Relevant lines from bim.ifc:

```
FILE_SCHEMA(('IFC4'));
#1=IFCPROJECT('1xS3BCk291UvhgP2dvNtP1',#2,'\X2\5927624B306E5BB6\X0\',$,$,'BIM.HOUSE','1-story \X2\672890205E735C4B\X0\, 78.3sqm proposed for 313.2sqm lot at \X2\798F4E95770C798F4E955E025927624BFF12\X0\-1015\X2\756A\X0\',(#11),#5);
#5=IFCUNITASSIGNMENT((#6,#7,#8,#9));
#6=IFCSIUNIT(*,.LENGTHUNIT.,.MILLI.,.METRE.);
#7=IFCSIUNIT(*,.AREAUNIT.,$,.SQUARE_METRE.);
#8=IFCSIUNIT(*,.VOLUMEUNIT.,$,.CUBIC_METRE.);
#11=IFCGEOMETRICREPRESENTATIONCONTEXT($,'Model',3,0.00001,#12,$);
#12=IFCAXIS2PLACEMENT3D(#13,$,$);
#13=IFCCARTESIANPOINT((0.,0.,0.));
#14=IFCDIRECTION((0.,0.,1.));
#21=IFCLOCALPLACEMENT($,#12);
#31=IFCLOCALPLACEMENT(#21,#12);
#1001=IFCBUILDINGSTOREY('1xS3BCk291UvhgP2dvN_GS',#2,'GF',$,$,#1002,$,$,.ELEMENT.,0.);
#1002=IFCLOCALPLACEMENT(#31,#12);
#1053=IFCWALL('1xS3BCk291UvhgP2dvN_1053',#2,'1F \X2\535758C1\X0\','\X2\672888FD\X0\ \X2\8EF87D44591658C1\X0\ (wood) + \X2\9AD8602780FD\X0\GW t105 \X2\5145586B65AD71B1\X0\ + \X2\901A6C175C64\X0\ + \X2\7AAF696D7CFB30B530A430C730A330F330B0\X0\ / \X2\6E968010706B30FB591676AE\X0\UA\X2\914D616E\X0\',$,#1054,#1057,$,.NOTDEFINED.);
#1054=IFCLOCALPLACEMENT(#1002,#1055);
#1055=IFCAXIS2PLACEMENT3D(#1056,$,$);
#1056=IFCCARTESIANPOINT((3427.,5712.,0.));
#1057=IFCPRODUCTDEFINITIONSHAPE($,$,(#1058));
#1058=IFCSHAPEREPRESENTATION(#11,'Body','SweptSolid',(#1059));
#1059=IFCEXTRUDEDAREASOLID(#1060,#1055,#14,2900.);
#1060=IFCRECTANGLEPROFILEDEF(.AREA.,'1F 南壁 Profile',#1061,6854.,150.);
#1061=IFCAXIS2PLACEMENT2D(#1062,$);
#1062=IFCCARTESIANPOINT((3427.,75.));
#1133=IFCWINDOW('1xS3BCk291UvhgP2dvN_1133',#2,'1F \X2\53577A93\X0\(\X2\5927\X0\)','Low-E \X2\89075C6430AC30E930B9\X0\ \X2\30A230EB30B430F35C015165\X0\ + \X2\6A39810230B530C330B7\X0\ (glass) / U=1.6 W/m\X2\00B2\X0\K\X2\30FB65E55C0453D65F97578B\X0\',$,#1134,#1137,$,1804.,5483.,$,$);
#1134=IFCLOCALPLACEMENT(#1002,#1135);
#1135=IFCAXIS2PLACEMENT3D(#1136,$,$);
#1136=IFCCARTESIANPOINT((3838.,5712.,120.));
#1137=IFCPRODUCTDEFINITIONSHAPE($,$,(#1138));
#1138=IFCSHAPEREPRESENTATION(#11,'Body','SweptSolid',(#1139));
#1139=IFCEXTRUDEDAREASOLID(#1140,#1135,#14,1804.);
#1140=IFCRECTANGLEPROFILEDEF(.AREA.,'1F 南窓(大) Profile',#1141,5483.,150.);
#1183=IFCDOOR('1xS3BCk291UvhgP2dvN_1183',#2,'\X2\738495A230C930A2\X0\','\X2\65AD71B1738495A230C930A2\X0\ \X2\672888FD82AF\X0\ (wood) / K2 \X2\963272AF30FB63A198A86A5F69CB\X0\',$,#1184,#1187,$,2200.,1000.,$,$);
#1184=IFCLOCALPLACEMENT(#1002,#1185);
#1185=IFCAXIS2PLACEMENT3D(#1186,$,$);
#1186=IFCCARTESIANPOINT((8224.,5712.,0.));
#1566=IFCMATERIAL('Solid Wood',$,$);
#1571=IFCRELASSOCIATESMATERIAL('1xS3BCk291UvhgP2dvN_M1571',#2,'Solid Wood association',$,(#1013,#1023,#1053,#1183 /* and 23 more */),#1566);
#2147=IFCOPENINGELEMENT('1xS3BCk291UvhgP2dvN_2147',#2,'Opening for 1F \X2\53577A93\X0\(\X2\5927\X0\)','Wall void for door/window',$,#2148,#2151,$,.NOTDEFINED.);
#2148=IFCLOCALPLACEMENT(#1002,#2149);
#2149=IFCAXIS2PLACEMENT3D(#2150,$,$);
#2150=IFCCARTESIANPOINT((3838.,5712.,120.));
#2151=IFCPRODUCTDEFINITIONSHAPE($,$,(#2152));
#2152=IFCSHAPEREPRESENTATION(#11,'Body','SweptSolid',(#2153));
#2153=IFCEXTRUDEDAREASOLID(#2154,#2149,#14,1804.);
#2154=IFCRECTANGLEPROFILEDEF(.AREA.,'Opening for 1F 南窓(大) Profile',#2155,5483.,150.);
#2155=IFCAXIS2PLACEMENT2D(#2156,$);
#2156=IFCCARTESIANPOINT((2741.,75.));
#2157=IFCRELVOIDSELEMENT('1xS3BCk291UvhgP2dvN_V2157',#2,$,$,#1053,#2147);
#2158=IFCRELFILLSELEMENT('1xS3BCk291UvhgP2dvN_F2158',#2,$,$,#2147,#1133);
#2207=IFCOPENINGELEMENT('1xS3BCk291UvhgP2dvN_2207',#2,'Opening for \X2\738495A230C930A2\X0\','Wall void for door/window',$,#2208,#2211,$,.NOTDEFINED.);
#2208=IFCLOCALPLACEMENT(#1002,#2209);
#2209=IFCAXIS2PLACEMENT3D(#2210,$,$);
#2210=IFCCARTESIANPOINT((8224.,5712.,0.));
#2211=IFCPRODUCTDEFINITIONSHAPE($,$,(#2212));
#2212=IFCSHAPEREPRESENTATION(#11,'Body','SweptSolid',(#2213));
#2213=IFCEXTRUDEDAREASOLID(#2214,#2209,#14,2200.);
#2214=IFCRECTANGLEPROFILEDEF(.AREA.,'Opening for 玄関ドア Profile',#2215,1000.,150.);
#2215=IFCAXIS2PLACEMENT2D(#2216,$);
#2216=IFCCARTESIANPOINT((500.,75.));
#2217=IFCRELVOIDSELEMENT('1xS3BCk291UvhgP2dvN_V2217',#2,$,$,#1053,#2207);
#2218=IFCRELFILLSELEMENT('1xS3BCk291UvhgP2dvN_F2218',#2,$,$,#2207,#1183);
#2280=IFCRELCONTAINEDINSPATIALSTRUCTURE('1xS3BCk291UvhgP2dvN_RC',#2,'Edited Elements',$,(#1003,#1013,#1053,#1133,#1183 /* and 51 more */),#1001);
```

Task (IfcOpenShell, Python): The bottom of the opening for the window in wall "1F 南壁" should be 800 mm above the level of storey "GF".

```python
import numpy as np
import ifcopenshell
import ifcopenshell.api.geometry
import ifcopenshell.geom
import ifcopenshell.util.element
import ifcopenshell.util.placement
import ifcopenshell.util.shape
import ifcopenshell.util.unit

model = ifcopenshell.open("bim.ifc")
unit_scale = ifcopenshell.util.unit.calculate_unit_scale(model)

window = model.by_guid("1xS3BCk291UvhgP2dvN_1133")
opening = window.FillsVoids[0].RelatingOpeningElement
storey = ifcopenshell.util.element.get_container(window, ifc_class="IfcBuildingStorey")
level = ifcopenshell.util.placement.get_local_placement(storey.ObjectPlacement)[2, 3]

# The opening's origin need not be at the sill, so measure its lowest point.
shape = ifcopenshell.geom.create_shape(ifcopenshell.geom.settings(), opening)
bottom = ifcopenshell.util.shape.get_shape_bottom_elevation(shape, shape.geometry) / unit_scale
dz = level + 0.8 / unit_scale - bottom

shift = np.array([0.0, 0.0, dz])
# The window is not placed relative to its opening, so move both.
for product in (opening, window):
    matrix = ifcopenshell.util.placement.get_local_placement(product.ObjectPlacement)
    matrix[:3, 3] += shift
    ifcopenshell.api.geometry.edit_object_placement(model, product=product, matrix=matrix, is_si=False)

print(f"moved by {dz * unit_scale:+.3f} m")

model.write("bim-out.ifc")
```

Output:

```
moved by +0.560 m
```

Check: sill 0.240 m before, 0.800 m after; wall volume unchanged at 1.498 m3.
